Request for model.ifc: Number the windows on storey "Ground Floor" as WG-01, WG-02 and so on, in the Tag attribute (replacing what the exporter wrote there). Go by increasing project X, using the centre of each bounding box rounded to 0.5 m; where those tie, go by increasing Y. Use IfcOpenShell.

First a look at what the model holds.

```python
import ifcopenshell
import ifcopenshell.util.element
import ifcopenshell.util.placement

model = ifcopenshell.open("model.ifc")
print(model.schema)
storey = next(s for s in model.by_type("IfcBuildingStorey") if s.Name == "Ground Floor")
windows = [e for e in ifcopenshell.util.element.get_decomposition(storey) if e.is_a("IfcWindow")]
for e in sorted(windows, key=lambda e: e.id()):
    origin = ifcopenshell.util.placement.get_local_placement(e.ObjectPlacement)[:3, 3]
    print(e.id(), e.Tag, e.Name, origin.round(2) + 0.0, sep=" | ")
```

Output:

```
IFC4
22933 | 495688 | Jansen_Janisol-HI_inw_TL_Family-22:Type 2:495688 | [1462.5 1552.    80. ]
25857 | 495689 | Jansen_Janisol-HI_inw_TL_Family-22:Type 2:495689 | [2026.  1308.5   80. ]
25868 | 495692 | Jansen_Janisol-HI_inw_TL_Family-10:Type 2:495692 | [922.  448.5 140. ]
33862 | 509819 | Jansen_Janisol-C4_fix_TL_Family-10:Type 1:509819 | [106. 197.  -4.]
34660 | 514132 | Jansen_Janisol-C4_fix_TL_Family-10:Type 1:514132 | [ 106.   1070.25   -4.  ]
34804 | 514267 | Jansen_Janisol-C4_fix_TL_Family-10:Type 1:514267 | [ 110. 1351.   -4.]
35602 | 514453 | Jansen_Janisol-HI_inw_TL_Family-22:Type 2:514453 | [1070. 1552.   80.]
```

```python
import ifcopenshell
import ifcopenshell.geom
import ifcopenshell.util.element
import ifcopenshell.util.shape

model = ifcopenshell.open("model.ifc")
settings = ifcopenshell.geom.settings()
settings.set("use-world-coords", True)


def centre(element):
    shape = ifcopenshell.geom.create_shape(settings, element)
    return ifcopenshell.util.shape.get_bbox_centroid(shape.geometry)


storey = next(s for s in model.by_type("IfcBuildingStorey") if s.Name == "Ground Floor")
windows = [e for e in ifcopenshell.util.element.get_decomposition(storey) if e.is_a("IfcWindow")]

# Insertion points can sit at a corner or the storey origin, so sort by the geometry (in metres).
centres = {e: centre(e) for e in windows}
windows.sort(key=lambda e: (round(centres[e][0] / 0.5), centres[e][1]))

for i, e in enumerate(windows, start=1):
    number = f"WG-{i:02d}"
    e.Tag = number
    print(e.id(), number)

model.write("model_updated.ifc")
```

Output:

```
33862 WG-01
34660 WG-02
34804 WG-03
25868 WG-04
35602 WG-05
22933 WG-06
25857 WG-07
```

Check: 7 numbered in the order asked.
